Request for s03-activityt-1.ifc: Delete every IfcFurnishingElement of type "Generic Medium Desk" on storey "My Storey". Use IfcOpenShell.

First a look at what the model holds.

```python
import ifcopenshell
import ifcopenshell.util.element

model = ifcopenshell.open("s03-activityt-1.ifc")
print(model.schema)
storey = next(s for s in model.by_type("IfcBuildingStorey") if s.Name == "My Storey")
furniture = [e for e in ifcopenshell.util.element.get_decomposition(storey) if e.is_a("IfcFurnishingElement")]
seen = {}
for e in furniture:
    element_type = ifcopenshell.util.element.get_type(e)
    name = element_type.Name if element_type not in (None, e) else None
    seen[name] = seen.get(name, 0) + 1
for name, count in sorted(seen.items(), key=str):
    print(count, "x", name)
```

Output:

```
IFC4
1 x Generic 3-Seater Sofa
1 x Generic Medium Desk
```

```python
import ifcopenshell
import ifcopenshell.api.root
import ifcopenshell.util.element

model = ifcopenshell.open("s03-activityt-1.ifc")

storey = next(s for s in model.by_type("IfcBuildingStorey") if s.Name == "My Storey")
furniture = [e for e in ifcopenshell.util.element.get_decomposition(storey) if e.is_a("IfcFurnishingElement")]
targets = [e for e in furniture if (t := ifcopenshell.util.element.get_type(e)) not in (None, e) and t.Name == "Generic Medium Desk"]

for e in targets:
    ifcopenshell.api.root.remove_product(model, product=e)
print(len(targets), "removed")

model.write("s03-activityt-1_updated.ifc")
```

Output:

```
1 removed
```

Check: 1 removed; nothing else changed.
